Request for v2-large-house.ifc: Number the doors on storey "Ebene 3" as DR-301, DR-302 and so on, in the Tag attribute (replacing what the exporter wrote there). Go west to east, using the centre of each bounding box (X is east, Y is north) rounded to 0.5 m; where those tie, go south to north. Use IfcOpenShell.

First a look at what the model holds.

```python
import ifcopenshell
import ifcopenshell.util.element
import ifcopenshell.util.placement

model = ifcopenshell.open("v2-large-house.ifc")
print(model.schema)
storey = next(s for s in model.by_type("IfcBuildingStorey") if s.Name == "Ebene 3")
doors = [e for e in ifcopenshell.util.element.get_decomposition(storey) if e.is_a("IfcDoor")]
for e in sorted(doors, key=lambda e: e.id()):
    origin = ifcopenshell.util.placement.get_local_placement(e.ObjectPlacement)[:3, 3]
    print(e.id(), e.Tag, e.Name, origin.round(2) + 0.0, sep=" | ")
```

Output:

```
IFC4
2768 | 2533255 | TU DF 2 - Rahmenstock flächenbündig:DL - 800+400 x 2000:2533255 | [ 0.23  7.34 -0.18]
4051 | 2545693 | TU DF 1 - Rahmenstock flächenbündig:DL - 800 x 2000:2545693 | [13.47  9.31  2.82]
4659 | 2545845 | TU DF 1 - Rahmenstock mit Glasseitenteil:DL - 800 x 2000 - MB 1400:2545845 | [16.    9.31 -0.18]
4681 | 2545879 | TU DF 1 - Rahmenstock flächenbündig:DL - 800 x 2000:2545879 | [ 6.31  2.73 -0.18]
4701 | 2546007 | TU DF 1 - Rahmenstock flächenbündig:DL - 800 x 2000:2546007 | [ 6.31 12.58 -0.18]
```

```python
import ifcopenshell
import ifcopenshell.geom
import ifcopenshell.util.element
import ifcopenshell.util.shape

model = ifcopenshell.open("v2-large-house.ifc")
settings = ifcopenshell.geom.settings()
settings.set("use-world-coords", True)


def centre(element):
    shape = ifcopenshell.geom.create_shape(settings, element)
    return ifcopenshell.util.shape.get_bbox_centroid(shape.geometry)


storey = next(s for s in model.by_type("IfcBuildingStorey") if s.Name == "Ebene 3")
doors = [e for e in ifcopenshell.util.element.get_decomposition(storey) if e.is_a("IfcDoor")]

# Insertion points can sit at a corner or the storey origin, so sort by the geometry (in metres).
centres = {e: centre(e) for e in doors}
doors.sort(key=lambda e: (round(centres[e][0] / 0.5), centres[e][1]))

for i, e in enumerate(doors, start=1):
    number = f"DR-3{i:02d}"
    e.Tag = number
    print(e.id(), number)

model.write("v2-large-house_edited.ifc")
```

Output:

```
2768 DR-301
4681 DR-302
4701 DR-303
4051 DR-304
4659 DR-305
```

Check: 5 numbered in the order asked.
